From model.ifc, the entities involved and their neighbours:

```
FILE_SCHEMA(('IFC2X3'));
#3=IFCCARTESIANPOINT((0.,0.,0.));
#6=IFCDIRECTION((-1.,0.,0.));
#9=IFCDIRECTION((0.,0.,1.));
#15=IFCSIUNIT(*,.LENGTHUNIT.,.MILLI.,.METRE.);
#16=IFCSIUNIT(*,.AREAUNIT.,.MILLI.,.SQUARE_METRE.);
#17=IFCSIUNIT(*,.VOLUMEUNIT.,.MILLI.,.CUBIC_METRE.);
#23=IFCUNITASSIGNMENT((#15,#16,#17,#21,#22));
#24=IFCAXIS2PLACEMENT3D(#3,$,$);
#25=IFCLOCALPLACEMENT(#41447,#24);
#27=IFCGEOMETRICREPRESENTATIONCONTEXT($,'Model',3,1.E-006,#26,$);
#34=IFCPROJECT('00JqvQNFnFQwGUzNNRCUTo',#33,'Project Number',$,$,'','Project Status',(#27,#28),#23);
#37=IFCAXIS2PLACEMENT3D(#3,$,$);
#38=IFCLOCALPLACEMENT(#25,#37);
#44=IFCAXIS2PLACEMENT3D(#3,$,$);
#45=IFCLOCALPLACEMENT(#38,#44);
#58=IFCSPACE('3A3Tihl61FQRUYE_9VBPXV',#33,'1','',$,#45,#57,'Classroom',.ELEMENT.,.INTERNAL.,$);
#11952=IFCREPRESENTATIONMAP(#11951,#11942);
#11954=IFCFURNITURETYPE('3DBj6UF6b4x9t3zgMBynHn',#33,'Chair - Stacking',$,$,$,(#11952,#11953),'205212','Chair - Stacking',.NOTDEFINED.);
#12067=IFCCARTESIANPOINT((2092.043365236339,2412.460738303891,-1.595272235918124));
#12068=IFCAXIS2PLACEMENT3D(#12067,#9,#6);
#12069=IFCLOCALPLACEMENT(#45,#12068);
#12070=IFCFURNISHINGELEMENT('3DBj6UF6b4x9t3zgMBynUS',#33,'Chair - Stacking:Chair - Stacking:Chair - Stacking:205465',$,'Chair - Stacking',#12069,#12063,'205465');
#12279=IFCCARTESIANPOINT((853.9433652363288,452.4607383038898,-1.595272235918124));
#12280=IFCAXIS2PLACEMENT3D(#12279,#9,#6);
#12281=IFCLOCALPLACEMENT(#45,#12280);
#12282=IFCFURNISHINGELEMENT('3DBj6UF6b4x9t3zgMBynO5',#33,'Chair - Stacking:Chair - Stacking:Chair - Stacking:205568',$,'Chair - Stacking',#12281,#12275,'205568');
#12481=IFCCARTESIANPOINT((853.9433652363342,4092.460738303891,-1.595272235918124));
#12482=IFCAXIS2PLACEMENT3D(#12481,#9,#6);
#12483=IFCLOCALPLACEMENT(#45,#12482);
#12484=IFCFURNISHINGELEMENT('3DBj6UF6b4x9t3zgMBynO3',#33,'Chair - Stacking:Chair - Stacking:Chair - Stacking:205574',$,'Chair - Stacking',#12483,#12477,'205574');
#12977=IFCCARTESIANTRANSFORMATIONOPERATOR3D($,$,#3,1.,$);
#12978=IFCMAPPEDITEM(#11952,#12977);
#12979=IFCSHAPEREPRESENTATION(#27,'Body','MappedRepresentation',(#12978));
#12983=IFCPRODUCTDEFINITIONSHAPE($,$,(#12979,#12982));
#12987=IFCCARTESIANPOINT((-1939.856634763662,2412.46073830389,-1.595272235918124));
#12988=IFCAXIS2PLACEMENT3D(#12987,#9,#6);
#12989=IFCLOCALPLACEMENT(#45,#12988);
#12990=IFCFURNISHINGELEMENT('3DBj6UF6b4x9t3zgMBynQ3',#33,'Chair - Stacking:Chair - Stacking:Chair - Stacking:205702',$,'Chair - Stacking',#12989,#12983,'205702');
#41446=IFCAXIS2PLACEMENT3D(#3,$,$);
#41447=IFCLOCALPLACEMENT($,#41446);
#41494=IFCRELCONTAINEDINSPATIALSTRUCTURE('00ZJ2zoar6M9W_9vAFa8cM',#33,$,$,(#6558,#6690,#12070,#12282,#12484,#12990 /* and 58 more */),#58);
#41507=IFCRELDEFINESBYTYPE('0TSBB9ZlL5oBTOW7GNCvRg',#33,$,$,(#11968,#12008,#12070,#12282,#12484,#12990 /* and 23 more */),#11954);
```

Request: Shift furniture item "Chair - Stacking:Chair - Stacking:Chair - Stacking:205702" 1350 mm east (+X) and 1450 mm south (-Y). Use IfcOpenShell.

```python
import ifcopenshell
import ifcopenshell.api.geometry
import ifcopenshell.util.placement
import ifcopenshell.util.unit

model = ifcopenshell.open("model.ifc")
unit_scale = ifcopenshell.util.unit.calculate_unit_scale(model)

item = model.by_guid("3DBj6UF6b4x9t3zgMBynQ3")
matrix = ifcopenshell.util.placement.get_local_placement(item.ObjectPlacement)
matrix[0, 3] += 1.35 / unit_scale
matrix[1, 3] -= 1.45 / unit_scale
ifcopenshell.api.geometry.edit_object_placement(model, product=item, matrix=matrix, is_si=False)

print(ifcopenshell.util.placement.get_local_placement(item.ObjectPlacement).round(3) + 0.0)

model.write("model_v2.ifc")
```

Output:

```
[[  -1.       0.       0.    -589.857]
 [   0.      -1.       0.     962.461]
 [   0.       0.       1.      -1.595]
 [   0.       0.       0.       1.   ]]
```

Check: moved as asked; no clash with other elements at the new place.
